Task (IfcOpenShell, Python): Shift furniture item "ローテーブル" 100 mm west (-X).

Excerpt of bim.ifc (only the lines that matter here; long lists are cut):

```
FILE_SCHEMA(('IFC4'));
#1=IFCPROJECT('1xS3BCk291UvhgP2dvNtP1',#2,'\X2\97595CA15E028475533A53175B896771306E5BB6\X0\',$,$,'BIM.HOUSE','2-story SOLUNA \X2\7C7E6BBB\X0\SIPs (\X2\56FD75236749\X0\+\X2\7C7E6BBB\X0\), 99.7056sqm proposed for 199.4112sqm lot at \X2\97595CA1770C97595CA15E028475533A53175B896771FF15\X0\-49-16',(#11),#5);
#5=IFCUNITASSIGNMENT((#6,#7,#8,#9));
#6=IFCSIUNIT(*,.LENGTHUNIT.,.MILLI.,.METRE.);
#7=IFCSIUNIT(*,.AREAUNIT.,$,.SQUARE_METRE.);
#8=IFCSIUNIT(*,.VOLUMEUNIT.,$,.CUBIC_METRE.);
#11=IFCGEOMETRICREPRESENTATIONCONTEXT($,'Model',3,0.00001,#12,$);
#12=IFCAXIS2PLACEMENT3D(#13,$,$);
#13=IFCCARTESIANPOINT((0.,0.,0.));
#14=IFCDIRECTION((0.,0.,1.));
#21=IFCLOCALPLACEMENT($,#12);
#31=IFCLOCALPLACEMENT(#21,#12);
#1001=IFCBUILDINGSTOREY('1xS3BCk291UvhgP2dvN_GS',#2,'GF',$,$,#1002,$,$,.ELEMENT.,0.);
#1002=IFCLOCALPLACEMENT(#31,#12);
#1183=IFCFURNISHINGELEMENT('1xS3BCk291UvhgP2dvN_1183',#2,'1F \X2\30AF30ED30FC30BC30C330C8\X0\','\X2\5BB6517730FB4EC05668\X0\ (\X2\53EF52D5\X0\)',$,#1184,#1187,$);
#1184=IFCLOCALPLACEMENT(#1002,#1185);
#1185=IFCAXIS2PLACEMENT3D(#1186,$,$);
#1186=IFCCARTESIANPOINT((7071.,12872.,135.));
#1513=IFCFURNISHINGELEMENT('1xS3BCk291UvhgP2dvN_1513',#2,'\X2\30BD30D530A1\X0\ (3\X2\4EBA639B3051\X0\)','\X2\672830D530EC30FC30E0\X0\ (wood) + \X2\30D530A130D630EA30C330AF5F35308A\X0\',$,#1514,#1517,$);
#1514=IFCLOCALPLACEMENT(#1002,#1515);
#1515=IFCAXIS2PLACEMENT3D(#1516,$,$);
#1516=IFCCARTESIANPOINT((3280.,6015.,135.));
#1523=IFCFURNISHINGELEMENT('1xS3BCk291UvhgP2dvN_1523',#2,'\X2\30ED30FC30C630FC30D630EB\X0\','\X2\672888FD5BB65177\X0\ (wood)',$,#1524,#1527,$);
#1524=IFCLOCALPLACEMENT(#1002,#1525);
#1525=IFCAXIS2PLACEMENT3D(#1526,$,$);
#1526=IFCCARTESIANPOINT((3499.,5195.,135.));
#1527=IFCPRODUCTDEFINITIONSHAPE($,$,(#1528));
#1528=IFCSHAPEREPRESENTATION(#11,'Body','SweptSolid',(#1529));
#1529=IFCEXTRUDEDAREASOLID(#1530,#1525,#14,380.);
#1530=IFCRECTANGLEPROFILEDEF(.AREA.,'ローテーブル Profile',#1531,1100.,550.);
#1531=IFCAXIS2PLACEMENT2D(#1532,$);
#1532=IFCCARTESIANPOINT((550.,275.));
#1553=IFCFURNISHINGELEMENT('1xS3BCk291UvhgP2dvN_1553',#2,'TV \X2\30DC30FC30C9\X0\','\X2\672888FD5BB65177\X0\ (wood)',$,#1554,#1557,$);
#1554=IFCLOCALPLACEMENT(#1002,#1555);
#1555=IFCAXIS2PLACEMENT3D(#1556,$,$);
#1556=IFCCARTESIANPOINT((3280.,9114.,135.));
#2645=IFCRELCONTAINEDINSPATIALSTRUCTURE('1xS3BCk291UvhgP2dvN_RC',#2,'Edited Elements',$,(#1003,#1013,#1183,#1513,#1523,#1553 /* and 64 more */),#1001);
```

```python
import ifcopenshell
import ifcopenshell.api.geometry
import ifcopenshell.util.placement
import ifcopenshell.util.unit

model = ifcopenshell.open("bim.ifc")
unit_scale = ifcopenshell.util.unit.calculate_unit_scale(model)

item = model.by_guid("1xS3BCk291UvhgP2dvN_1523")
matrix = ifcopenshell.util.placement.get_local_placement(item.ObjectPlacement)
matrix[0, 3] -= 0.1 / unit_scale
ifcopenshell.api.geometry.edit_object_placement(model, product=item, matrix=matrix, is_si=False)

print(ifcopenshell.util.placement.get_local_placement(item.ObjectPlacement).round(3) + 0.0)

model.write("bim_v2.ifc")
```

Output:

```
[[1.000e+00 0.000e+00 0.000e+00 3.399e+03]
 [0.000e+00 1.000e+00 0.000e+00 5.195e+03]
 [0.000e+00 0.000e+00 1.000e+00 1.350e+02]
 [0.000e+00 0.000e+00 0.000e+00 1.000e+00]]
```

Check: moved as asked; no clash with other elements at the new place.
